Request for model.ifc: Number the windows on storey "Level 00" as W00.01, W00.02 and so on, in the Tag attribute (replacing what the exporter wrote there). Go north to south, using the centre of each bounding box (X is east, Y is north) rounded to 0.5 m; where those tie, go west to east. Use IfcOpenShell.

First a look at what the model holds.

```python
import ifcopenshell
import ifcopenshell.util.element
import ifcopenshell.util.placement

model = ifcopenshell.open("model.ifc")
print(model.schema)
storey = next(s for s in model.by_type("IfcBuildingStorey") if s.Name == "Level 00")
windows = [e for e in ifcopenshell.util.element.get_decomposition(storey) if e.is_a("IfcWindow")]
for e in sorted(windows, key=lambda e: e.id()):
    origin = ifcopenshell.util.placement.get_local_placement(e.ObjectPlacement)[:3, 3]
    print(e.id(), e.Tag, e.Name, origin.round(2) + 0.0, sep=" | ")
```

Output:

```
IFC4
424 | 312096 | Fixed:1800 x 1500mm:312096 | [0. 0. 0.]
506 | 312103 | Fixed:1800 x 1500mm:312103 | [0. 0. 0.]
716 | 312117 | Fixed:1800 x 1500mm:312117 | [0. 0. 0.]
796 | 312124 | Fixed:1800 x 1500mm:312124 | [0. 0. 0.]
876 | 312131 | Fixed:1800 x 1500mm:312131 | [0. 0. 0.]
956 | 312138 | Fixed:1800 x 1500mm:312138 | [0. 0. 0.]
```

```python
import ifcopenshell
import ifcopenshell.geom
import ifcopenshell.util.element
import ifcopenshell.util.shape

model = ifcopenshell.open("model.ifc")
settings = ifcopenshell.geom.settings()
settings.set("use-world-coords", True)


def centre(element):
    shape = ifcopenshell.geom.create_shape(settings, element)
    return ifcopenshell.util.shape.get_bbox_centroid(shape.geometry)


storey = next(s for s in model.by_type("IfcBuildingStorey") if s.Name == "Level 00")
windows = [e for e in ifcopenshell.util.element.get_decomposition(storey) if e.is_a("IfcWindow")]

# Insertion points can sit at a corner or the storey origin, so sort by the geometry (in metres).
centres = {e: centre(e) for e in windows}
windows.sort(key=lambda e: (-round(centres[e][1] / 0.5), centres[e][0]))

for i, e in enumerate(windows, start=1):
    number = f"W00.{i:02d}"
    e.Tag = number
    print(e.id(), number)

model.write("model-out.ifc")
```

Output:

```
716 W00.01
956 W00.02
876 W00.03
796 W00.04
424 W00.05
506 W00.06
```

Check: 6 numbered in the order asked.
